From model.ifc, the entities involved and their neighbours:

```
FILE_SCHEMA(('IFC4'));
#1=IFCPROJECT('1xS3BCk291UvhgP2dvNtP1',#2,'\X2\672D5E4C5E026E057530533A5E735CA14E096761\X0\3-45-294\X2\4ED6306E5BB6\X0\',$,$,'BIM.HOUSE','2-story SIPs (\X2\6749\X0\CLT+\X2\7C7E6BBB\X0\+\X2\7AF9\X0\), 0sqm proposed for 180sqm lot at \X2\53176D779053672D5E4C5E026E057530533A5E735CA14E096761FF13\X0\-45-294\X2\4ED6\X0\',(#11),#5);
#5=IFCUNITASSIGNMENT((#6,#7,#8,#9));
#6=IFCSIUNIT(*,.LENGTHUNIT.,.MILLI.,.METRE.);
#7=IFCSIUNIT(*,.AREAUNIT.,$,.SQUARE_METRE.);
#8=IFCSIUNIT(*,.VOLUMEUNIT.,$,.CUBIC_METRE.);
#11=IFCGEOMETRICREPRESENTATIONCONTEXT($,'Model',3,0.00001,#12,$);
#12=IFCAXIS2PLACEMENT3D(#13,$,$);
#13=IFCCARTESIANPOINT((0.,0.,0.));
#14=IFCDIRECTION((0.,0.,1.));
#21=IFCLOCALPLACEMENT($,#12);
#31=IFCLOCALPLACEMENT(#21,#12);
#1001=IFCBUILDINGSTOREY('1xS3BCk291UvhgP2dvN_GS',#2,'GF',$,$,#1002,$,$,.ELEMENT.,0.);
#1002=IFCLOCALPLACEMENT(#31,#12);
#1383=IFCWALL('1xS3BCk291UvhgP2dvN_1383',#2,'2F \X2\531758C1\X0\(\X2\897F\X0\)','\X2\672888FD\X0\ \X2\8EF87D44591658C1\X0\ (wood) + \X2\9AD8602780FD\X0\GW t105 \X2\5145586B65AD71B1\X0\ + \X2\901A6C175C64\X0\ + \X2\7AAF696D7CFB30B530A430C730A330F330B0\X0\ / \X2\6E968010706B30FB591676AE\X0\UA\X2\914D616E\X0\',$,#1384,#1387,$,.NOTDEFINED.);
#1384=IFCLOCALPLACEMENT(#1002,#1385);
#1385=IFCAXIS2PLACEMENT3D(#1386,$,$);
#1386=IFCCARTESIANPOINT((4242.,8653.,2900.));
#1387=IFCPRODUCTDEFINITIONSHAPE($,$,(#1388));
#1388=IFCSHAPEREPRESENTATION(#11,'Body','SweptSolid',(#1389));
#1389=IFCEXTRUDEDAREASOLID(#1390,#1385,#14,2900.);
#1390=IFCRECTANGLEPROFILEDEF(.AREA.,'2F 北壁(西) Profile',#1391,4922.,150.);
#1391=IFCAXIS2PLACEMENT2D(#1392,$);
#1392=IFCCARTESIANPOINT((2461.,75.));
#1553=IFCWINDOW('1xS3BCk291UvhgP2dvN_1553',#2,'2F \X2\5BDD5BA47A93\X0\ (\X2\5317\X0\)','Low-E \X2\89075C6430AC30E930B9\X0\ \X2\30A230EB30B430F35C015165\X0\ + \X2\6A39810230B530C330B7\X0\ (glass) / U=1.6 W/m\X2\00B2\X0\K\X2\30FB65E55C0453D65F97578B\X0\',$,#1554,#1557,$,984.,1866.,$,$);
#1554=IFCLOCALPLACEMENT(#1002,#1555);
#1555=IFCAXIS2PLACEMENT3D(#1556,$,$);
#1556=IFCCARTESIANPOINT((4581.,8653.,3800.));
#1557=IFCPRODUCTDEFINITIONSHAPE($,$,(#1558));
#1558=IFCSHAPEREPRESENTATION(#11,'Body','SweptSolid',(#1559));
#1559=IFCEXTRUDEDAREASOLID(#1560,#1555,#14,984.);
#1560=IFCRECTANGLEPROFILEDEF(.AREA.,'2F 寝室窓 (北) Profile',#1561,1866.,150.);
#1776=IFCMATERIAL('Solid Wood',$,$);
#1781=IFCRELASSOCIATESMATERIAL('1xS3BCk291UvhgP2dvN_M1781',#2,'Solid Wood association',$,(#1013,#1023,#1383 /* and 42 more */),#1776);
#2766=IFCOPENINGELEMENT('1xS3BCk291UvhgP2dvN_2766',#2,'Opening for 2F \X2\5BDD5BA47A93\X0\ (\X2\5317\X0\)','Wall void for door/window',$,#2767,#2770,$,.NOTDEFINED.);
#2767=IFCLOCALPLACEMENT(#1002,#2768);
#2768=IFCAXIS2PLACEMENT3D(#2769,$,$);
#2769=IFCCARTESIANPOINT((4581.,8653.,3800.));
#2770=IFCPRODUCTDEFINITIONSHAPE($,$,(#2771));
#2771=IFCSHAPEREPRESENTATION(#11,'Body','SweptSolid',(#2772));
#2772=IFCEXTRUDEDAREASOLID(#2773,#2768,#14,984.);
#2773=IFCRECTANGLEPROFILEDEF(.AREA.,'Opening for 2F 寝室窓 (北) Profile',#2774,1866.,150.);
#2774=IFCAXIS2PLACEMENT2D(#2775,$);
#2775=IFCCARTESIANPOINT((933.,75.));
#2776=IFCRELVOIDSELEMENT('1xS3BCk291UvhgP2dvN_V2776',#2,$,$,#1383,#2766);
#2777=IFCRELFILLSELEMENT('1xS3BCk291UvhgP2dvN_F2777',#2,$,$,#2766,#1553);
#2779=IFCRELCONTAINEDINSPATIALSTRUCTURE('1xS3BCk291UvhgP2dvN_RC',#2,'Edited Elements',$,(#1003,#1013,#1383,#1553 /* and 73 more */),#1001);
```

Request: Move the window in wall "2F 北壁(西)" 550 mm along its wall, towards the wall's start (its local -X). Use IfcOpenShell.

```python
import ifcopenshell
import ifcopenshell.api.geometry
import ifcopenshell.util.placement

model = ifcopenshell.open("model.ifc")

window = model.by_guid("1xS3BCk291UvhgP2dvN_1553")
opening = window.FillsVoids[0].RelatingOpeningElement
wall = opening.VoidsElements[0].RelatingBuildingElement

wall_matrix = ifcopenshell.util.placement.get_local_placement(wall.ObjectPlacement)
shift = wall_matrix[:3, 0] * -550.0
before = ifcopenshell.util.placement.get_local_placement(window.ObjectPlacement)[:3, 3].copy()

# The window is not placed relative to its opening, so move both.
for product in (opening, window):
    matrix = ifcopenshell.util.placement.get_local_placement(product.ObjectPlacement)
    matrix[:3, 3] += shift
    ifcopenshell.api.geometry.edit_object_placement(model, product=product, matrix=matrix, is_si=False)

after = ifcopenshell.util.placement.get_local_placement(window.ObjectPlacement)[:3, 3]
print("window moved by", (after - before).round(3) + 0.0)

model.write("model_updated.ifc")
```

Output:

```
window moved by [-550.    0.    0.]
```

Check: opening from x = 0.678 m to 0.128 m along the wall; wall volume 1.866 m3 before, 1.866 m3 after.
